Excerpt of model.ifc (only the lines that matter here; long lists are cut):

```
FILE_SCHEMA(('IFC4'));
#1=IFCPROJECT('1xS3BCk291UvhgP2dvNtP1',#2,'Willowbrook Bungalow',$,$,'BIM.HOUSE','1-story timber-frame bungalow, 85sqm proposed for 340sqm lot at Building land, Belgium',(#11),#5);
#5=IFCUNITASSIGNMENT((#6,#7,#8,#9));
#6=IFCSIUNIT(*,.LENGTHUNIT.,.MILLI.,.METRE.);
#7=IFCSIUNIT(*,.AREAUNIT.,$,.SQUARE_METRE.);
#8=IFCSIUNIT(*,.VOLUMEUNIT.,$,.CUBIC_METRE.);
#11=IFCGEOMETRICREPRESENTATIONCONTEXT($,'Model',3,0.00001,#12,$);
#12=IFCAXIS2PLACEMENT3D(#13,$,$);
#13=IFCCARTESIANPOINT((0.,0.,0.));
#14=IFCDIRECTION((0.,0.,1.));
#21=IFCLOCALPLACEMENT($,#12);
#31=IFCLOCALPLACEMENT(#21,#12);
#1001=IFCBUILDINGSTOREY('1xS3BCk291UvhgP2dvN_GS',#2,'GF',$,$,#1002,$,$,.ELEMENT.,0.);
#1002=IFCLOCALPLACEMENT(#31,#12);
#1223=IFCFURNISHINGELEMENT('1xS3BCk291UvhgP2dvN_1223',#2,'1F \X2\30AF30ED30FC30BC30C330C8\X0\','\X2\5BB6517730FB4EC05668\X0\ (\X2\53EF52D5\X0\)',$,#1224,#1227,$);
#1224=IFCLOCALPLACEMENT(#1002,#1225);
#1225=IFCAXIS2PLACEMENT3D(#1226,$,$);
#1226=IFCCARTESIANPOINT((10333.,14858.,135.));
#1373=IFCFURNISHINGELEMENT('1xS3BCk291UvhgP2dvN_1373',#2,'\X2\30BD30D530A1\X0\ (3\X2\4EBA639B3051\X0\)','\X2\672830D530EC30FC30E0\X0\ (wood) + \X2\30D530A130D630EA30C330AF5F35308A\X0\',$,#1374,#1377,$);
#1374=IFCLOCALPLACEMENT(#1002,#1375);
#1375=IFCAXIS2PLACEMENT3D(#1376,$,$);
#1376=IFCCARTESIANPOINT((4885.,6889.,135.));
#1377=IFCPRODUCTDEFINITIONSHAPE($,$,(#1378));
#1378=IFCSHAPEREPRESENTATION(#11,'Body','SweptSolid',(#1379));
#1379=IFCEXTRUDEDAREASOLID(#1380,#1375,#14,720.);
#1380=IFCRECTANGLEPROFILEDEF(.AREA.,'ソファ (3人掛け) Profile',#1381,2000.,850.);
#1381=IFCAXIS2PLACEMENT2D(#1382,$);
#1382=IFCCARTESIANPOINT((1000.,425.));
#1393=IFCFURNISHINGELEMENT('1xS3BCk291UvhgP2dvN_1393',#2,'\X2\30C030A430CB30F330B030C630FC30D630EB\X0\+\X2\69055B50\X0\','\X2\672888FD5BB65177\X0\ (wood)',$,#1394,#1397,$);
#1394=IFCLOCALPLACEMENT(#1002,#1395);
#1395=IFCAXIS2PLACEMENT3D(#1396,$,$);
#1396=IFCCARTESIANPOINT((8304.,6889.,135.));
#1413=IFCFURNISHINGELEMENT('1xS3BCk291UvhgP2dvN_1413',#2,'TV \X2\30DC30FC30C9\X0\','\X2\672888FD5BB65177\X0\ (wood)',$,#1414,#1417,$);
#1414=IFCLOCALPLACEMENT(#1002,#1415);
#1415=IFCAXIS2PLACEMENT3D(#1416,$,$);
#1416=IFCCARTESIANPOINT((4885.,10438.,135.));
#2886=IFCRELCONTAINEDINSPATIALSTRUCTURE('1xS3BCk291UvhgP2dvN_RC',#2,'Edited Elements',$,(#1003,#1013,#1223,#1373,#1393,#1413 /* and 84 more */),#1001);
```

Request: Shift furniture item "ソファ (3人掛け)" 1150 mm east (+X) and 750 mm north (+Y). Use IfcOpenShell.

```python
import ifcopenshell
import ifcopenshell.api.geometry
import ifcopenshell.util.placement

model = ifcopenshell.open("model.ifc")

item = model.by_guid("1xS3BCk291UvhgP2dvN_1373")
matrix = ifcopenshell.util.placement.get_local_placement(item.ObjectPlacement)
matrix[0, 3] += 1150.0
matrix[1, 3] += 750.0
ifcopenshell.api.geometry.edit_object_placement(model, product=item, matrix=matrix, is_si=False)

print(ifcopenshell.util.placement.get_local_placement(item.ObjectPlacement).round(3) + 0.0)

model.write("model-out.ifc")
```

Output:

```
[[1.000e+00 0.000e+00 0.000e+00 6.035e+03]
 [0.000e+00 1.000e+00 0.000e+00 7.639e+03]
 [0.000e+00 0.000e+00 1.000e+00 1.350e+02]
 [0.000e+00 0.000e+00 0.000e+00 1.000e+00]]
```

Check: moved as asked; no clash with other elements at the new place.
